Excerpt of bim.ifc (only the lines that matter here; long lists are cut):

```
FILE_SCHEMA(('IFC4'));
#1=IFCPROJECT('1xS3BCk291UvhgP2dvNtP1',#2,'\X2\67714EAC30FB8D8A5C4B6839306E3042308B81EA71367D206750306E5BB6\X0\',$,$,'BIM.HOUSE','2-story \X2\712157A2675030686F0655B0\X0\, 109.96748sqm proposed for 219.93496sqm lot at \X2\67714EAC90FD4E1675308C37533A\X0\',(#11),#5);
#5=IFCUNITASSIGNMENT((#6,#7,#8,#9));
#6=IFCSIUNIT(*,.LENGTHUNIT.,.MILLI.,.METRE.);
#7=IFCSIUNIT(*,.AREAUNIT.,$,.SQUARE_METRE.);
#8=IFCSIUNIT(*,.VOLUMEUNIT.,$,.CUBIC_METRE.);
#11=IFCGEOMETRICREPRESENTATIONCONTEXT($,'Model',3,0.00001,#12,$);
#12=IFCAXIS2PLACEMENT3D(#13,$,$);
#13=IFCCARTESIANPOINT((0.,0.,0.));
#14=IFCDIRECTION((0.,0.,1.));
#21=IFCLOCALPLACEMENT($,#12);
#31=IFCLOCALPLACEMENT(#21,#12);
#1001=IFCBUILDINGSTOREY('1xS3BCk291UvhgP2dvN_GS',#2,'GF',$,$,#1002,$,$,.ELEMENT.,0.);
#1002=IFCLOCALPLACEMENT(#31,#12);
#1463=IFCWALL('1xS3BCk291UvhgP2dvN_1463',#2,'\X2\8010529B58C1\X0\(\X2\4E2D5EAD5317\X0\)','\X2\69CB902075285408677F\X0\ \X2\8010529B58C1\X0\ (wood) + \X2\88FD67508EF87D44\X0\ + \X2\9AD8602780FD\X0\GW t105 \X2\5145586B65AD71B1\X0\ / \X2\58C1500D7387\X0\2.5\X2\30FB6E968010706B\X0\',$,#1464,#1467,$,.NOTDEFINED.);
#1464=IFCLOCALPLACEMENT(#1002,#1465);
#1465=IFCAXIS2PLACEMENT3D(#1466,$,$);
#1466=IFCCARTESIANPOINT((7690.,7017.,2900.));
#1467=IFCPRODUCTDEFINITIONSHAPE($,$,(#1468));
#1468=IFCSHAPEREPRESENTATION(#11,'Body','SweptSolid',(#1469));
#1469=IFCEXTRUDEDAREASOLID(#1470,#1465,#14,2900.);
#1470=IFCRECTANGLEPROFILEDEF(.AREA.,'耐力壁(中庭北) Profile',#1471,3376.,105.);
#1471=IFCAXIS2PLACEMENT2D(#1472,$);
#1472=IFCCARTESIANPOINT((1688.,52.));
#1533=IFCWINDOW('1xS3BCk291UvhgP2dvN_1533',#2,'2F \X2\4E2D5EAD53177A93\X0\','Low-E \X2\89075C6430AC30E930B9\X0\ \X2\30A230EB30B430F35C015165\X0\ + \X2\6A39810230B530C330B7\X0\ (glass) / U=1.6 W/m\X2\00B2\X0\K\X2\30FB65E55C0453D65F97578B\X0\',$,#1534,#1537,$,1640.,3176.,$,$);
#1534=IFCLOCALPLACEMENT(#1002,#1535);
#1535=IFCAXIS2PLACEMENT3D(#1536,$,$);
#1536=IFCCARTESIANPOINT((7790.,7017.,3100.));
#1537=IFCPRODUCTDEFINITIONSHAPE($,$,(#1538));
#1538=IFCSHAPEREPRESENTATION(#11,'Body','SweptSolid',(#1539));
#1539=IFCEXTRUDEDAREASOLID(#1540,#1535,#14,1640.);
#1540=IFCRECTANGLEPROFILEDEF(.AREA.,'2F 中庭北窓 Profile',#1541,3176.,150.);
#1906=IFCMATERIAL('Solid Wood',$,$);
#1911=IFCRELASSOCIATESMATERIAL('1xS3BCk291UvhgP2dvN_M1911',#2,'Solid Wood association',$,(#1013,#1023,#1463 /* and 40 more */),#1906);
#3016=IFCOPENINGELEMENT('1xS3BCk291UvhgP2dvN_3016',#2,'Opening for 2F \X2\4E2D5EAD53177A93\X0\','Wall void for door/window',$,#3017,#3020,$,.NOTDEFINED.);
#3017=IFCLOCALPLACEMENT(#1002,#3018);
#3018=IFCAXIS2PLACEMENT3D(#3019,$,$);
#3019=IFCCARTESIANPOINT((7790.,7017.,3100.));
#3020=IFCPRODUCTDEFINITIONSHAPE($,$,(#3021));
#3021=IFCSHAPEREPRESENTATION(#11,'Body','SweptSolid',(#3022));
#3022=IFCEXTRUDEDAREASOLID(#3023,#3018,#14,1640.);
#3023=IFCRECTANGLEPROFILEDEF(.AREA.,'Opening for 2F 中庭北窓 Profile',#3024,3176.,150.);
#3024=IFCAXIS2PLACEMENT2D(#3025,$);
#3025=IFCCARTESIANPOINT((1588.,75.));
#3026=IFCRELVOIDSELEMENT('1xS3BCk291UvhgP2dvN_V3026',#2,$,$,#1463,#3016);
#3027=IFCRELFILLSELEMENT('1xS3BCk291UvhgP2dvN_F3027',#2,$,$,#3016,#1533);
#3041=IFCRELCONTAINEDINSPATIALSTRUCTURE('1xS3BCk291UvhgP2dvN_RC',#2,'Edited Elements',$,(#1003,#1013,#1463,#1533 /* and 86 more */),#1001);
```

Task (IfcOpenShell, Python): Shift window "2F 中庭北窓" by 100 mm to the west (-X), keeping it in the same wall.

```python
import ifcopenshell
import ifcopenshell.api.geometry
import ifcopenshell.util.placement
import ifcopenshell.util.unit

model = ifcopenshell.open("bim.ifc")
unit_scale = ifcopenshell.util.unit.calculate_unit_scale(model)

window = model.by_id(1533)
opening = window.FillsVoids[0].RelatingOpeningElement
wall = opening.VoidsElements[0].RelatingBuildingElement

wall_matrix = ifcopenshell.util.placement.get_local_placement(wall.ObjectPlacement)
shift = wall_matrix[:3, 0] * -0.1 / unit_scale
before = ifcopenshell.util.placement.get_local_placement(window.ObjectPlacement)[:3, 3].copy()

# The window is not placed relative to its opening, so move both.
for product in (opening, window):
    matrix = ifcopenshell.util.placement.get_local_placement(product.ObjectPlacement)
    matrix[:3, 3] += shift
    ifcopenshell.api.geometry.edit_object_placement(model, product=product, matrix=matrix, is_si=False)

after = ifcopenshell.util.placement.get_local_placement(window.ObjectPlacement)[:3, 3]
print("window moved by", (after - before).round(3) + 0.0)

model.write("bim_edited.ifc")
```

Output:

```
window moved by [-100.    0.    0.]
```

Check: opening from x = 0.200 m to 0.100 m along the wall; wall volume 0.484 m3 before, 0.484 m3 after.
